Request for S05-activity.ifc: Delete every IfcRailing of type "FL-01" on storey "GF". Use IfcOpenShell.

First a look at what the model holds.

```python
import ifcopenshell
import ifcopenshell.util.element

model = ifcopenshell.open("S05-activity.ifc")
print(model.schema)
storey = next(s for s in model.by_type("IfcBuildingStorey") if s.Name == "GF")
railings = [e for e in ifcopenshell.util.element.get_decomposition(storey) if e.is_a("IfcRailing")]
seen = {}
for e in railings:
    element_type = ifcopenshell.util.element.get_type(e)
    name = element_type.Name if element_type not in (None, e) else None
    seen[name] = seen.get(name, 0) + 1
for name, count in sorted(seen.items(), key=str):
    print(count, "x", name)
```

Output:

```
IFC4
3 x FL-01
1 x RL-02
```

```python
import ifcopenshell
import ifcopenshell.api.root
import ifcopenshell.util.element

model = ifcopenshell.open("S05-activity.ifc")

storey = next(s for s in model.by_type("IfcBuildingStorey") if s.Name == "GF")
railings = [e for e in ifcopenshell.util.element.get_decomposition(storey) if e.is_a("IfcRailing")]
targets = [e for e in railings if (t := ifcopenshell.util.element.get_type(e)) not in (None, e) and t.Name == "FL-01"]

for e in targets:
    ifcopenshell.api.root.remove_product(model, product=e)
print(len(targets), "removed")

model.write("S05-activity_v2.ifc")
```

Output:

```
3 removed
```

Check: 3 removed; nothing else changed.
